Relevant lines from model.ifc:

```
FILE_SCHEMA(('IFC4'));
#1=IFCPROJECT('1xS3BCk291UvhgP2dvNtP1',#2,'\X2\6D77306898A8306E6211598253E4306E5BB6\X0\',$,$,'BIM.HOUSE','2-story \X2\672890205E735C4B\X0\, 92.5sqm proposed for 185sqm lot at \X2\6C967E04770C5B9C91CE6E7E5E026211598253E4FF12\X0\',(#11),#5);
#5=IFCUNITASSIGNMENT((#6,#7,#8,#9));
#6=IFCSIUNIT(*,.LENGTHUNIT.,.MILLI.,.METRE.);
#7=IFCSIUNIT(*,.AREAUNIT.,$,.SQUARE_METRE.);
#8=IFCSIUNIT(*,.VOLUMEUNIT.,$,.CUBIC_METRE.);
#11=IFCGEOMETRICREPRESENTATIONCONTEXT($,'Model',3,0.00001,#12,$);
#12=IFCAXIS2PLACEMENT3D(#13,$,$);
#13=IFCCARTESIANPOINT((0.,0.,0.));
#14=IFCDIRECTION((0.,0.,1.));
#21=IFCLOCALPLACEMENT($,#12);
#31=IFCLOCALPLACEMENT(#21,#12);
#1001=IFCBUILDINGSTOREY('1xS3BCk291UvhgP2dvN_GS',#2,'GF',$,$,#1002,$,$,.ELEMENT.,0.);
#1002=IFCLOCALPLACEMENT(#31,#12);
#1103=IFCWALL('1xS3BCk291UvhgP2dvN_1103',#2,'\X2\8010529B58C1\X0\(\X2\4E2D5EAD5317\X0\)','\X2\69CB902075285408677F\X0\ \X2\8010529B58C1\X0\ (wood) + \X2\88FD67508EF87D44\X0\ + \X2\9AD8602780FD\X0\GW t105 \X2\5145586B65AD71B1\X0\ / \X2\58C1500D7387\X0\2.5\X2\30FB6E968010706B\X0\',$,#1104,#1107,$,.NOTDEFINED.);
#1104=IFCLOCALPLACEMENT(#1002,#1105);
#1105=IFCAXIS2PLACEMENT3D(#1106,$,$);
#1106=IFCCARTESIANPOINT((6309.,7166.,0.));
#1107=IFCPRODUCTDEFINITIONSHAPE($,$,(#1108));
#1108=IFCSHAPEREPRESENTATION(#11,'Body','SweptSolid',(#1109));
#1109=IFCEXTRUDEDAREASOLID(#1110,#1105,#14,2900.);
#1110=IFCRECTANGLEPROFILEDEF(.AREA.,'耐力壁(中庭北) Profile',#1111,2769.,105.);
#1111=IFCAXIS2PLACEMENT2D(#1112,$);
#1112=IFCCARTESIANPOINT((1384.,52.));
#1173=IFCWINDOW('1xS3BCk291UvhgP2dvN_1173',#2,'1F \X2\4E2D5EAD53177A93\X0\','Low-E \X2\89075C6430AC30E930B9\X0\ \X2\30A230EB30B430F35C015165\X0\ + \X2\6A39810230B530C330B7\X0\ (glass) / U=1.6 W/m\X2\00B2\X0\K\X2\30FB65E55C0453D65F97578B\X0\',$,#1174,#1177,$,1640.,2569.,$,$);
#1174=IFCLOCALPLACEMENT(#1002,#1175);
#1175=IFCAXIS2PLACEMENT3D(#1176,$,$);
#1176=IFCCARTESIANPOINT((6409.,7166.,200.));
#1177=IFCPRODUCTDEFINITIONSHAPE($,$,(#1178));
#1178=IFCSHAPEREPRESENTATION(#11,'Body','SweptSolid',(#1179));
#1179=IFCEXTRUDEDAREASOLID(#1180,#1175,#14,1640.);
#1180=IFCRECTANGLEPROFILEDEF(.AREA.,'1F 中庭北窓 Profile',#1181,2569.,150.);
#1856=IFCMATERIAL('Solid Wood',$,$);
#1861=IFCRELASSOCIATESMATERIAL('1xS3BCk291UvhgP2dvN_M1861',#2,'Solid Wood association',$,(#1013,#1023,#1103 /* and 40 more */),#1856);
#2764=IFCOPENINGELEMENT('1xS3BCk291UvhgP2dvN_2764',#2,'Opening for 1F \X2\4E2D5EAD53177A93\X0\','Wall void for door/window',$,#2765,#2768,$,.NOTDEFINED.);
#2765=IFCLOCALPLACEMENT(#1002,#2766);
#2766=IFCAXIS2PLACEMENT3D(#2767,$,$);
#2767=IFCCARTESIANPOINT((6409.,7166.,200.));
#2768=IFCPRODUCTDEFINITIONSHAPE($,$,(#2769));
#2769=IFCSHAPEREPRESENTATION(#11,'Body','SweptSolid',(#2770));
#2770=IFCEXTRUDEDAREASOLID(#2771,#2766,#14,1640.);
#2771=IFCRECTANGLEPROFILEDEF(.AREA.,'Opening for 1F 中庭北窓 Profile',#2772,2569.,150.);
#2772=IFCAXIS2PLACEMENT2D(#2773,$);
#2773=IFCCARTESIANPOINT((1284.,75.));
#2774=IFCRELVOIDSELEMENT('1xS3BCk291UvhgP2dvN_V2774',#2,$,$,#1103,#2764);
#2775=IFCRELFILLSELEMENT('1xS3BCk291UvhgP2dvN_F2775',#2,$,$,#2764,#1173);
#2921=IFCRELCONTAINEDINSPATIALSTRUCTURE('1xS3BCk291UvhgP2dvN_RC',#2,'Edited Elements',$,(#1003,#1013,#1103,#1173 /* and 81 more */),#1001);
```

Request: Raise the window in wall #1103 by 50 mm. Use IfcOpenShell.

```python
import numpy as np
import ifcopenshell
import ifcopenshell.api.geometry
import ifcopenshell.util.placement
import ifcopenshell.util.unit

model = ifcopenshell.open("model.ifc")
unit_scale = ifcopenshell.util.unit.calculate_unit_scale(model)

window = model.by_id(1173)
opening = window.FillsVoids[0].RelatingOpeningElement
dz = 0.05 / unit_scale

shift = np.array([0.0, 0.0, dz])
# The window is not placed relative to its opening, so move both.
for product in (opening, window):
    matrix = ifcopenshell.util.placement.get_local_placement(product.ObjectPlacement)
    matrix[:3, 3] += shift
    ifcopenshell.api.geometry.edit_object_placement(model, product=product, matrix=matrix, is_si=False)

print(f"moved by {dz * unit_scale:+.3f} m")

model.write("model_rev.ifc")
```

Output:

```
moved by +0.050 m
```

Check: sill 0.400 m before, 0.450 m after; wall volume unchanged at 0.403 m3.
